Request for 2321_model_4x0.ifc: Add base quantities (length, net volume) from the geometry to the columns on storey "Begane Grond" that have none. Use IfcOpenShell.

First a look at what the model holds.

```python
import ifcopenshell
import ifcopenshell.util.element
import ifcopenshell.util.unit

model = ifcopenshell.open("2321_model_4x0.ifc")
print(model.schema)
for unit_type in ("LENGTHUNIT", "AREAUNIT", "VOLUMEUNIT"):
    print(unit_type, ifcopenshell.util.unit.calculate_unit_scale(model, unit_type))
storey = next(s for s in model.by_type("IfcBuildingStorey") if s.Name == "Begane Grond")
columns = [e for e in ifcopenshell.util.element.get_decomposition(storey) if e.is_a("IfcColumn")]
for e in sorted(columns, key=lambda e: e.id()):
    print(e.id(), e.is_a(), e.Name, list(ifcopenshell.util.element.get_psets(e, qtos_only=True)), sep=" | ")
```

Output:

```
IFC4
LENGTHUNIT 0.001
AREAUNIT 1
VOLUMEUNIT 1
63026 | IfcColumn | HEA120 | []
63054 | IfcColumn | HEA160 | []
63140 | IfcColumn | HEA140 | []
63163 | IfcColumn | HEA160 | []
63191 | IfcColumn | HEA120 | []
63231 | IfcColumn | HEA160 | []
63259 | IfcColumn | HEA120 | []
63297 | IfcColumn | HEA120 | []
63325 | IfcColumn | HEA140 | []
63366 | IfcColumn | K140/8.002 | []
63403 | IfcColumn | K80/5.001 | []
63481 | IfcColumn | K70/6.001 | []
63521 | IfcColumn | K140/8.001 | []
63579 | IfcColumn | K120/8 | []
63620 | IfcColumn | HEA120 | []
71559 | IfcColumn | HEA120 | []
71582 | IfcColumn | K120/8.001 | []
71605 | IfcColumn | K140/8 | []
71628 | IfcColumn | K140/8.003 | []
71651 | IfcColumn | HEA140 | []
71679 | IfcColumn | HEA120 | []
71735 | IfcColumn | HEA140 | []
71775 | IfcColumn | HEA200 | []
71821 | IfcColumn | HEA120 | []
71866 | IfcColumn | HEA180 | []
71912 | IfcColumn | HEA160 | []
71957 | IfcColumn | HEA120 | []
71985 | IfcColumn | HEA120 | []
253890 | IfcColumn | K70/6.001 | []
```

```python
import ifcopenshell
import ifcopenshell.api.pset
import ifcopenshell.geom
import ifcopenshell.util.element
import ifcopenshell.util.shape
import ifcopenshell.util.unit

model = ifcopenshell.open("2321_model_4x0.ifc")
unit_scale = ifcopenshell.util.unit.calculate_unit_scale(model)
volume_scale = ifcopenshell.util.unit.calculate_unit_scale(model, "VOLUMEUNIT")
settings = ifcopenshell.geom.settings()

storey = next(s for s in model.by_type("IfcBuildingStorey") if s.Name == "Begane Grond")
columns = [e for e in ifcopenshell.util.element.get_decomposition(storey) if e.is_a("IfcColumn")]

for e in sorted(columns, key=lambda e: e.id()):
    if ifcopenshell.util.element.get_psets(e, qtos_only=True, should_inherit=False):
        continue
    # Geometry comes back in metres, in the element's own axes.
    shape = ifcopenshell.geom.create_shape(settings, e)
    values = {
        "Length": ifcopenshell.util.shape.get_z(shape.geometry) / unit_scale,
        "NetVolume": ifcopenshell.util.shape.get_volume(shape.geometry) / volume_scale,
    }
    qto = ifcopenshell.api.pset.add_qto(model, product=e, name="Qto_ColumnBaseQuantities")
    ifcopenshell.api.pset.edit_qto(model, qto=qto, properties=values)
    print(e.id(), {k: round(v, 3) for k, v in values.items()})

model.write("2321_model_4x0_edited.ifc")
```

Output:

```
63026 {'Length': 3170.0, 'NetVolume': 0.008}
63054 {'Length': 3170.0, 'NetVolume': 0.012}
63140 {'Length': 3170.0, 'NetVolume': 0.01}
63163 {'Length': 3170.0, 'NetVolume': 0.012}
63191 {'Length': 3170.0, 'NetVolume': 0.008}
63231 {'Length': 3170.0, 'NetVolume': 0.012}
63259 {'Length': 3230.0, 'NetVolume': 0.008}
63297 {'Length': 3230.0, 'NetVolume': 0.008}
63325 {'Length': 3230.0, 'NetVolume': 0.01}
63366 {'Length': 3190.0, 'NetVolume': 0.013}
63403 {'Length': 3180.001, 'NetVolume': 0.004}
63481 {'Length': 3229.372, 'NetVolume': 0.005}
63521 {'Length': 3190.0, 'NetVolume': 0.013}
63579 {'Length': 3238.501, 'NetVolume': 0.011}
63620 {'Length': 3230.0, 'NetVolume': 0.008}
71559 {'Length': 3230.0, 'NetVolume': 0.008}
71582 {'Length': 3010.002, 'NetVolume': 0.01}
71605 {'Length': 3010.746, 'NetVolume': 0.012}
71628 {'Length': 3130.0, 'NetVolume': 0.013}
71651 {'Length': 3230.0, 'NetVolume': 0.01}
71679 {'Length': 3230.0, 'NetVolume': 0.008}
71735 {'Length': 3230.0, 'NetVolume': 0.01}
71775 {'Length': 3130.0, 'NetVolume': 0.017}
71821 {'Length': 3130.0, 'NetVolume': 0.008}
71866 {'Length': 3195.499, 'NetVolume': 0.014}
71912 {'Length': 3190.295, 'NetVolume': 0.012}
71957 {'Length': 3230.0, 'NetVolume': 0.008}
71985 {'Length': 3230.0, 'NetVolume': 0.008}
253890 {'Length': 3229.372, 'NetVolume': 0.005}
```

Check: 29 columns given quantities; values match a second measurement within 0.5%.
